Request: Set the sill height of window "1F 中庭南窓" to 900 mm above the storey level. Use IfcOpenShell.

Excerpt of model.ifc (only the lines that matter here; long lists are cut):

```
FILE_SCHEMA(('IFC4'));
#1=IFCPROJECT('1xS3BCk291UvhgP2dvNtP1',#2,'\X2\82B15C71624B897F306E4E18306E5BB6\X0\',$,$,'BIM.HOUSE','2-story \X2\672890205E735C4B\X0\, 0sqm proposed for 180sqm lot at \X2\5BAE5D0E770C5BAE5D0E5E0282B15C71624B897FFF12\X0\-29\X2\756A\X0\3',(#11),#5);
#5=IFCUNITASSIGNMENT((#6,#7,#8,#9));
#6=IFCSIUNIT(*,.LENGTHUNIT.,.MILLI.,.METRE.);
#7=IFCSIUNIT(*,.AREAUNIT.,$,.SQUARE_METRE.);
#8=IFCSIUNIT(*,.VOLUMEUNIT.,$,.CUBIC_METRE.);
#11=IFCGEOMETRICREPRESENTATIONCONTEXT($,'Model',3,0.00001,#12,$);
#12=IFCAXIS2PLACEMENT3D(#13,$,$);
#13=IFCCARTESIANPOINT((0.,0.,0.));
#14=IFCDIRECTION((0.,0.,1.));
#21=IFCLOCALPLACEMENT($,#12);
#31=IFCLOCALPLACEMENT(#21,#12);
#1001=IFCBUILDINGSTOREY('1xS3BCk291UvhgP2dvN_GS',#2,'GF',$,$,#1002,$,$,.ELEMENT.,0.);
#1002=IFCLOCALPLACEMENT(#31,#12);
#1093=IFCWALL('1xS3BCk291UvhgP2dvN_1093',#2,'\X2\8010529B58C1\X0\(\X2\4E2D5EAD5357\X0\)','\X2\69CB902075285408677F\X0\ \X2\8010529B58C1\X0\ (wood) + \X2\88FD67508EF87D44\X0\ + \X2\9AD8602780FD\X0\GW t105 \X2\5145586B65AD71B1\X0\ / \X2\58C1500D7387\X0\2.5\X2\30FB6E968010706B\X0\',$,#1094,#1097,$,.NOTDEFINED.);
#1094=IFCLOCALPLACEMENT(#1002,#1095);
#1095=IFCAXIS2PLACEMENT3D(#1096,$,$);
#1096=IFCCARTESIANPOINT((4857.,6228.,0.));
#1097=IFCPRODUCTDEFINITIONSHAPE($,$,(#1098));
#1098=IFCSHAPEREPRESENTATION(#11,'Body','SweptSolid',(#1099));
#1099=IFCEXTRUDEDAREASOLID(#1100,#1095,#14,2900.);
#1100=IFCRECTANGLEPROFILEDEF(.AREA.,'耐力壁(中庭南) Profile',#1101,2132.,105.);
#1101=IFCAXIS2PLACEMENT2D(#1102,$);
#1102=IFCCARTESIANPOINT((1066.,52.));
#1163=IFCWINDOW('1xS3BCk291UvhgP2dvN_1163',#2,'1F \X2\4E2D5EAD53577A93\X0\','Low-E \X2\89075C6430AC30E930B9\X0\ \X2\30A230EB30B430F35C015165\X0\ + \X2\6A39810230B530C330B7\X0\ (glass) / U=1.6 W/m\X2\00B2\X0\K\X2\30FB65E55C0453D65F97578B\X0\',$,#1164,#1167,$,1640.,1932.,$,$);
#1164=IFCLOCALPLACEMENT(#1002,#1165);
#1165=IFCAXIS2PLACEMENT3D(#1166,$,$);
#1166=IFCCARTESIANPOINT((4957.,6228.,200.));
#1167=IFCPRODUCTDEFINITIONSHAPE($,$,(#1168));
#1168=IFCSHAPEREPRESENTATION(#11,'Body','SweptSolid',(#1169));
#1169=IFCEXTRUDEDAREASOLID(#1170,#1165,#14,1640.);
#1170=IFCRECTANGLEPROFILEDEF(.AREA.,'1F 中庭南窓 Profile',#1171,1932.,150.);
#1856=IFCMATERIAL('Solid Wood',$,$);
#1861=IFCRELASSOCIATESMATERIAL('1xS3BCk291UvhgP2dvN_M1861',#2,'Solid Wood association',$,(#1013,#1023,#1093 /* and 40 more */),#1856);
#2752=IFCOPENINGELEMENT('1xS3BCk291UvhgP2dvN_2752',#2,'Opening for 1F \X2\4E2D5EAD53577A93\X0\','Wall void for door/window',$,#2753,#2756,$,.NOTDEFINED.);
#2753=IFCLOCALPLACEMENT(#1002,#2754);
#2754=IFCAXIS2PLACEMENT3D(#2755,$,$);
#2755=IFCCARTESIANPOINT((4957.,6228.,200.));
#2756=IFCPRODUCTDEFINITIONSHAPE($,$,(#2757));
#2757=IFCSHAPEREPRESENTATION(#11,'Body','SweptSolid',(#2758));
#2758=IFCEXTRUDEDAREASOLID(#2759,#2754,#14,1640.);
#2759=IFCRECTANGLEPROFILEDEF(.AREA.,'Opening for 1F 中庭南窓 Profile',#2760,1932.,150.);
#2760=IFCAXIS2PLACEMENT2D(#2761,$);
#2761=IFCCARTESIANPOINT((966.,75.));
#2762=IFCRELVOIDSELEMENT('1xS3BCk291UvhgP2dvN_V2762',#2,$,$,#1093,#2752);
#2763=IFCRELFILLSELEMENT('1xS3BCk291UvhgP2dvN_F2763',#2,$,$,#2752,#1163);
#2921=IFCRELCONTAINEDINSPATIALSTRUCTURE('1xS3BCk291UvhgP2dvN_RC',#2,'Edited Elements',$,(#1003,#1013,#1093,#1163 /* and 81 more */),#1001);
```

```python
import numpy as np
import ifcopenshell
import ifcopenshell.api.geometry
import ifcopenshell.geom
import ifcopenshell.util.element
import ifcopenshell.util.placement
import ifcopenshell.util.shape
import ifcopenshell.util.unit

model = ifcopenshell.open("model.ifc")
unit_scale = ifcopenshell.util.unit.calculate_unit_scale(model)

window = model.by_guid("1xS3BCk291UvhgP2dvN_1163")
opening = window.FillsVoids[0].RelatingOpeningElement
storey = ifcopenshell.util.element.get_container(window, ifc_class="IfcBuildingStorey")
level = ifcopenshell.util.placement.get_local_placement(storey.ObjectPlacement)[2, 3]

# The opening's origin need not be at the sill, so measure its lowest point.
shape = ifcopenshell.geom.create_shape(ifcopenshell.geom.settings(), opening)
bottom = ifcopenshell.util.shape.get_shape_bottom_elevation(shape, shape.geometry) / unit_scale
dz = level + 900.0 - bottom

shift = np.array([0.0, 0.0, dz])
# The window is not placed relative to its opening, so move both.
for product in (opening, window):
    matrix = ifcopenshell.util.placement.get_local_placement(product.ObjectPlacement)
    matrix[:3, 3] += shift
    ifcopenshell.api.geometry.edit_object_placement(model, product=product, matrix=matrix, is_si=False)

print(f"moved by {dz * unit_scale:+.3f} m")

model.write("model_rev.ifc")
```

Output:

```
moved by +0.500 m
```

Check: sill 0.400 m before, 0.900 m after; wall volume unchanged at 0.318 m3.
